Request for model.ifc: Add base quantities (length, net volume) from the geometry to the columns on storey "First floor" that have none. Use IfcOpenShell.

First a look at what the model holds.

```python
import ifcopenshell
import ifcopenshell.util.element
import ifcopenshell.util.unit

model = ifcopenshell.open("model.ifc")
print(model.schema)
for unit_type in ("LENGTHUNIT", "AREAUNIT", "VOLUMEUNIT"):
    print(unit_type, ifcopenshell.util.unit.calculate_unit_scale(model, unit_type))
storey = next(s for s in model.by_type("IfcBuildingStorey") if s.Name == "First floor")
columns = [e for e in ifcopenshell.util.element.get_decomposition(storey) if e.is_a("IfcColumn")]
for e in sorted(columns, key=lambda e: e.id()):
    print(e.id(), e.is_a(), e.Name, list(ifcopenshell.util.element.get_psets(e, qtos_only=True)), sep=" | ")
```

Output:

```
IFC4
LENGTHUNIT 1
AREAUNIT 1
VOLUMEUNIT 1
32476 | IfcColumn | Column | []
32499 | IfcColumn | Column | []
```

```python
import ifcopenshell
import ifcopenshell.api.pset
import ifcopenshell.geom
import ifcopenshell.util.element
import ifcopenshell.util.shape
import ifcopenshell.util.unit

model = ifcopenshell.open("model.ifc")
unit_scale = ifcopenshell.util.unit.calculate_unit_scale(model)
volume_scale = ifcopenshell.util.unit.calculate_unit_scale(model, "VOLUMEUNIT")
settings = ifcopenshell.geom.settings()

storey = next(s for s in model.by_type("IfcBuildingStorey") if s.Name == "First floor")
columns = [e for e in ifcopenshell.util.element.get_decomposition(storey) if e.is_a("IfcColumn")]

for e in sorted(columns, key=lambda e: e.id()):
    if ifcopenshell.util.element.get_psets(e, qtos_only=True, should_inherit=False):
        continue
    # Geometry comes back in metres, in the element's own axes.
    shape = ifcopenshell.geom.create_shape(settings, e)
    values = {
        "Length": ifcopenshell.util.shape.get_z(shape.geometry) / unit_scale,
        "NetVolume": ifcopenshell.util.shape.get_volume(shape.geometry) / volume_scale,
    }
    qto = ifcopenshell.api.pset.add_qto(model, product=e, name="Qto_ColumnBaseQuantities")
    ifcopenshell.api.pset.edit_qto(model, qto=qto, properties=values)
    print(e.id(), {k: round(v, 3) for k, v in values.items()})

model.write("model-out.ifc")
```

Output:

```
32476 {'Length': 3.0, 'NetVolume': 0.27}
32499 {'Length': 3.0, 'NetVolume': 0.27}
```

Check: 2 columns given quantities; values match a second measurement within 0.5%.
